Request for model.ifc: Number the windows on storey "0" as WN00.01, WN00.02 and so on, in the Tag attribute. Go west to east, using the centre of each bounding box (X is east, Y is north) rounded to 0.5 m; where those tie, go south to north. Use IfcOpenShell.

First a look at what the model holds.

```python
import ifcopenshell
import ifcopenshell.util.element
import ifcopenshell.util.placement

model = ifcopenshell.open("model.ifc")
print(model.schema)
storey = next(s for s in model.by_type("IfcBuildingStorey") if s.Name == "0")
windows = [e for e in ifcopenshell.util.element.get_decomposition(storey) if e.is_a("IfcWindow")]
for e in sorted(windows, key=lambda e: e.id()):
    origin = ifcopenshell.util.placement.get_local_placement(e.ObjectPlacement)[:3, 3]
    print(e.id(), e.Tag, e.Name, origin.round(2) + 0.0, sep=" | ")
```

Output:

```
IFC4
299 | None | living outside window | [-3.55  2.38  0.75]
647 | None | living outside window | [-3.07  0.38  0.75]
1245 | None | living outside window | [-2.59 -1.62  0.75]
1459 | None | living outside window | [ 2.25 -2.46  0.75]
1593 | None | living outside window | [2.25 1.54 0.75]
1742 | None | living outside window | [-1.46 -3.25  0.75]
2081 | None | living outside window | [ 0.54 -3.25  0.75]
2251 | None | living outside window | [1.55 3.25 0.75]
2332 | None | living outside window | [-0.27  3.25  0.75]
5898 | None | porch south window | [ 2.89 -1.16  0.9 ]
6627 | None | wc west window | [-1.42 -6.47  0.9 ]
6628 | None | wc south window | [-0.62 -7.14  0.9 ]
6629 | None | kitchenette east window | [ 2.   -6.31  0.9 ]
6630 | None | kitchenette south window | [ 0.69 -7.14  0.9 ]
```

```python
import ifcopenshell
import ifcopenshell.geom
import ifcopenshell.util.element
import ifcopenshell.util.shape

model = ifcopenshell.open("model.ifc")
settings = ifcopenshell.geom.settings()
settings.set("use-world-coords", True)


def centre(element):
    shape = ifcopenshell.geom.create_shape(settings, element)
    return ifcopenshell.util.shape.get_bbox_centroid(shape.geometry)


storey = next(s for s in model.by_type("IfcBuildingStorey") if s.Name == "0")
windows = [e for e in ifcopenshell.util.element.get_decomposition(storey) if e.is_a("IfcWindow")]

# Insertion points can sit at a corner or the storey origin, so sort by the geometry (in metres).
centres = {e: centre(e) for e in windows}
windows.sort(key=lambda e: (round(centres[e][0] / 0.5), centres[e][1]))

for i, e in enumerate(windows, start=1):
    number = f"WN00.{i:02d}"
    e.Tag = number
    print(e.id(), number)

model.write("model-out.ifc")
```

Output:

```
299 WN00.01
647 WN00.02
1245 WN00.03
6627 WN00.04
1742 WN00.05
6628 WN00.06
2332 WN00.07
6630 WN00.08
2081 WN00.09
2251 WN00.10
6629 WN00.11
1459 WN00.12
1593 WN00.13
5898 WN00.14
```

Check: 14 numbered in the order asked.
